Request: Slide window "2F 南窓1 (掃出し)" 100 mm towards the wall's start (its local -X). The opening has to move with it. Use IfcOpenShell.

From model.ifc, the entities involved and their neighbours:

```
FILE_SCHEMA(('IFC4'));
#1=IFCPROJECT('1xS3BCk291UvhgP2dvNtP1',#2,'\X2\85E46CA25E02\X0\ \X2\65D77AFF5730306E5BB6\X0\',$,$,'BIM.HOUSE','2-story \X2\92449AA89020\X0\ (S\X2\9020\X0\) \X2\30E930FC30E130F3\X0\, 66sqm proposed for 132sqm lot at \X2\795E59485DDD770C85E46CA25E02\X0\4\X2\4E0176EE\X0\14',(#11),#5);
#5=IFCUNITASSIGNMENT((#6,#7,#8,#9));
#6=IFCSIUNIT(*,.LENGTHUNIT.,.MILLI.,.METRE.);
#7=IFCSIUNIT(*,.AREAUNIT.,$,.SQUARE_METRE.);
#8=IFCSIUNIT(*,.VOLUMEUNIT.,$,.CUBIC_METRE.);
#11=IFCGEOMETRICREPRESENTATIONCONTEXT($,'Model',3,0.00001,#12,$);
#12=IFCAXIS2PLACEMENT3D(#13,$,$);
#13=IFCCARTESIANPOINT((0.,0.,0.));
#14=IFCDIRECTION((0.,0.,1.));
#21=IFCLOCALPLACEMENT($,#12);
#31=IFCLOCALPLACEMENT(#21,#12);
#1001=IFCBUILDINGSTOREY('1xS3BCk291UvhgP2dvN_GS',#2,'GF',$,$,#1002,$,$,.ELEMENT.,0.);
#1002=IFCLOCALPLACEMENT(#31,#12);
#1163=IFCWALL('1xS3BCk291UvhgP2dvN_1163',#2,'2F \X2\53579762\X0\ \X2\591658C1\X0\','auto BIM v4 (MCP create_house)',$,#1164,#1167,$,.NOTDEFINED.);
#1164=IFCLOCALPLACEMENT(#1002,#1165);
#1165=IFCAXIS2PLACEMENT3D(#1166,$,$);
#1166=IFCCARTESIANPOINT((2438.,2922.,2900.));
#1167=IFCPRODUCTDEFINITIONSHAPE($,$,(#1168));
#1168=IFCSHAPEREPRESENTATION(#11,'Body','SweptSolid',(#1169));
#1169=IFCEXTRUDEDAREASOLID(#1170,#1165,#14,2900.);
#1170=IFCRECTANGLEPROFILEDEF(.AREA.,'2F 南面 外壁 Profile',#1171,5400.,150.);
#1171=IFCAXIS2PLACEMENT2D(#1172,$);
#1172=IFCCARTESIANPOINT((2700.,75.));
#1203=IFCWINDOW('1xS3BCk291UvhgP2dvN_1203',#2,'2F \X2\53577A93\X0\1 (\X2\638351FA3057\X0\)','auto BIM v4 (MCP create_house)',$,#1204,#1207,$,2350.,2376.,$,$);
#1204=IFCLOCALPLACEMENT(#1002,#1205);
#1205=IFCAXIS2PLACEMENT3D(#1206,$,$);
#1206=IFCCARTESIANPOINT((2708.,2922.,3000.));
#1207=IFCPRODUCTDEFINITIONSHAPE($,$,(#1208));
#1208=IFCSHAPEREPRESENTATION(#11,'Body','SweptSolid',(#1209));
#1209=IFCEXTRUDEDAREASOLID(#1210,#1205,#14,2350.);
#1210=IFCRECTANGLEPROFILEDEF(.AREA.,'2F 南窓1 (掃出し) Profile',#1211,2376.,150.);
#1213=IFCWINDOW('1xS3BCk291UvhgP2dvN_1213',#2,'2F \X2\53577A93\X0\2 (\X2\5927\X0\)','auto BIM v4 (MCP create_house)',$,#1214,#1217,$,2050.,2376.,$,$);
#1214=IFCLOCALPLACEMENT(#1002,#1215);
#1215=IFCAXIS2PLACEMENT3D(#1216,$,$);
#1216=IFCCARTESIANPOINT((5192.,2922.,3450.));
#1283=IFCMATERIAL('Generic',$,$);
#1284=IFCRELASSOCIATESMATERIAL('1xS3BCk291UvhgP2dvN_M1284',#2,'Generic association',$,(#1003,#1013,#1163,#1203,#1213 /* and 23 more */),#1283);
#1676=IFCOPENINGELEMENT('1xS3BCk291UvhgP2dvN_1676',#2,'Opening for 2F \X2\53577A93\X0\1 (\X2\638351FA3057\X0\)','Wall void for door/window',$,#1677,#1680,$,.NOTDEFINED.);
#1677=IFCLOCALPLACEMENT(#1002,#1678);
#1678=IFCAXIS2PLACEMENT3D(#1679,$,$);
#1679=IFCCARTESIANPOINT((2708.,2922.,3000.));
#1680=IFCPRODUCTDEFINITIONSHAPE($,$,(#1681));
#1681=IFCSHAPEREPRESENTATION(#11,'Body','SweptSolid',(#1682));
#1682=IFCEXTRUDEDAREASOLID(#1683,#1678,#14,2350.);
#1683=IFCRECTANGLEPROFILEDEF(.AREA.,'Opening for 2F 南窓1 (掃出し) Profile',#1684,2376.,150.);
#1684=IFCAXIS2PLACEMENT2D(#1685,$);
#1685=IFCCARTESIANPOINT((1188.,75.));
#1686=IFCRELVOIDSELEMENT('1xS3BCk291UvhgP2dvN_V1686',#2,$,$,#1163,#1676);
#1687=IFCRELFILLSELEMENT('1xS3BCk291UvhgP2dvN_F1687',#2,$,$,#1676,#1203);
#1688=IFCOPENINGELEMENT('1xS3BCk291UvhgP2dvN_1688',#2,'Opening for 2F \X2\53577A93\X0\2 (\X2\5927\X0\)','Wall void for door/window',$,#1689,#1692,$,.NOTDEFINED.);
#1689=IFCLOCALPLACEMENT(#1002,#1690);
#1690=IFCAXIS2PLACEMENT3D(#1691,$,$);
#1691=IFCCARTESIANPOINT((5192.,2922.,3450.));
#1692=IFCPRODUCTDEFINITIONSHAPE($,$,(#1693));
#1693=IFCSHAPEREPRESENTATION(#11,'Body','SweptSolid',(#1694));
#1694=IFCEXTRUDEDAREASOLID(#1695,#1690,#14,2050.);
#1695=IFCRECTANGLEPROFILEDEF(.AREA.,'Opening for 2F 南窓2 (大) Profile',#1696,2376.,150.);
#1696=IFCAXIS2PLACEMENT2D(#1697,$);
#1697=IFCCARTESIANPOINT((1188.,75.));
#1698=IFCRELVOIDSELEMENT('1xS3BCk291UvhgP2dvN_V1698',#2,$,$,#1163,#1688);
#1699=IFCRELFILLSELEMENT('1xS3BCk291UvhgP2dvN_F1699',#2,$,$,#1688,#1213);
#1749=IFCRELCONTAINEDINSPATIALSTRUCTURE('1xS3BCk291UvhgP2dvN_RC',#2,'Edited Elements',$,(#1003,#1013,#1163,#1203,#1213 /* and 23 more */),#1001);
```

```python
import ifcopenshell
import ifcopenshell.api.geometry
import ifcopenshell.util.placement
import ifcopenshell.util.unit

model = ifcopenshell.open("model.ifc")
unit_scale = ifcopenshell.util.unit.calculate_unit_scale(model)

window = model.by_guid("1xS3BCk291UvhgP2dvN_1203")
opening = window.FillsVoids[0].RelatingOpeningElement
wall = opening.VoidsElements[0].RelatingBuildingElement

wall_matrix = ifcopenshell.util.placement.get_local_placement(wall.ObjectPlacement)
shift = wall_matrix[:3, 0] * -0.1 / unit_scale
before = ifcopenshell.util.placement.get_local_placement(window.ObjectPlacement)[:3, 3].copy()

# The window is not placed relative to its opening, so move both.
for product in (opening, window):
    matrix = ifcopenshell.util.placement.get_local_placement(product.ObjectPlacement)
    matrix[:3, 3] += shift
    ifcopenshell.api.geometry.edit_object_placement(model, product=product, matrix=matrix, is_si=False)

after = ifcopenshell.util.placement.get_local_placement(window.ObjectPlacement)[:3, 3]
print("window moved by", (after - before).round(3) + 0.0)

model.write("model_edited.ifc")
```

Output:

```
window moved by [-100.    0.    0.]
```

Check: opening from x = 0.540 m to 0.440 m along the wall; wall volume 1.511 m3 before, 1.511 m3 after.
